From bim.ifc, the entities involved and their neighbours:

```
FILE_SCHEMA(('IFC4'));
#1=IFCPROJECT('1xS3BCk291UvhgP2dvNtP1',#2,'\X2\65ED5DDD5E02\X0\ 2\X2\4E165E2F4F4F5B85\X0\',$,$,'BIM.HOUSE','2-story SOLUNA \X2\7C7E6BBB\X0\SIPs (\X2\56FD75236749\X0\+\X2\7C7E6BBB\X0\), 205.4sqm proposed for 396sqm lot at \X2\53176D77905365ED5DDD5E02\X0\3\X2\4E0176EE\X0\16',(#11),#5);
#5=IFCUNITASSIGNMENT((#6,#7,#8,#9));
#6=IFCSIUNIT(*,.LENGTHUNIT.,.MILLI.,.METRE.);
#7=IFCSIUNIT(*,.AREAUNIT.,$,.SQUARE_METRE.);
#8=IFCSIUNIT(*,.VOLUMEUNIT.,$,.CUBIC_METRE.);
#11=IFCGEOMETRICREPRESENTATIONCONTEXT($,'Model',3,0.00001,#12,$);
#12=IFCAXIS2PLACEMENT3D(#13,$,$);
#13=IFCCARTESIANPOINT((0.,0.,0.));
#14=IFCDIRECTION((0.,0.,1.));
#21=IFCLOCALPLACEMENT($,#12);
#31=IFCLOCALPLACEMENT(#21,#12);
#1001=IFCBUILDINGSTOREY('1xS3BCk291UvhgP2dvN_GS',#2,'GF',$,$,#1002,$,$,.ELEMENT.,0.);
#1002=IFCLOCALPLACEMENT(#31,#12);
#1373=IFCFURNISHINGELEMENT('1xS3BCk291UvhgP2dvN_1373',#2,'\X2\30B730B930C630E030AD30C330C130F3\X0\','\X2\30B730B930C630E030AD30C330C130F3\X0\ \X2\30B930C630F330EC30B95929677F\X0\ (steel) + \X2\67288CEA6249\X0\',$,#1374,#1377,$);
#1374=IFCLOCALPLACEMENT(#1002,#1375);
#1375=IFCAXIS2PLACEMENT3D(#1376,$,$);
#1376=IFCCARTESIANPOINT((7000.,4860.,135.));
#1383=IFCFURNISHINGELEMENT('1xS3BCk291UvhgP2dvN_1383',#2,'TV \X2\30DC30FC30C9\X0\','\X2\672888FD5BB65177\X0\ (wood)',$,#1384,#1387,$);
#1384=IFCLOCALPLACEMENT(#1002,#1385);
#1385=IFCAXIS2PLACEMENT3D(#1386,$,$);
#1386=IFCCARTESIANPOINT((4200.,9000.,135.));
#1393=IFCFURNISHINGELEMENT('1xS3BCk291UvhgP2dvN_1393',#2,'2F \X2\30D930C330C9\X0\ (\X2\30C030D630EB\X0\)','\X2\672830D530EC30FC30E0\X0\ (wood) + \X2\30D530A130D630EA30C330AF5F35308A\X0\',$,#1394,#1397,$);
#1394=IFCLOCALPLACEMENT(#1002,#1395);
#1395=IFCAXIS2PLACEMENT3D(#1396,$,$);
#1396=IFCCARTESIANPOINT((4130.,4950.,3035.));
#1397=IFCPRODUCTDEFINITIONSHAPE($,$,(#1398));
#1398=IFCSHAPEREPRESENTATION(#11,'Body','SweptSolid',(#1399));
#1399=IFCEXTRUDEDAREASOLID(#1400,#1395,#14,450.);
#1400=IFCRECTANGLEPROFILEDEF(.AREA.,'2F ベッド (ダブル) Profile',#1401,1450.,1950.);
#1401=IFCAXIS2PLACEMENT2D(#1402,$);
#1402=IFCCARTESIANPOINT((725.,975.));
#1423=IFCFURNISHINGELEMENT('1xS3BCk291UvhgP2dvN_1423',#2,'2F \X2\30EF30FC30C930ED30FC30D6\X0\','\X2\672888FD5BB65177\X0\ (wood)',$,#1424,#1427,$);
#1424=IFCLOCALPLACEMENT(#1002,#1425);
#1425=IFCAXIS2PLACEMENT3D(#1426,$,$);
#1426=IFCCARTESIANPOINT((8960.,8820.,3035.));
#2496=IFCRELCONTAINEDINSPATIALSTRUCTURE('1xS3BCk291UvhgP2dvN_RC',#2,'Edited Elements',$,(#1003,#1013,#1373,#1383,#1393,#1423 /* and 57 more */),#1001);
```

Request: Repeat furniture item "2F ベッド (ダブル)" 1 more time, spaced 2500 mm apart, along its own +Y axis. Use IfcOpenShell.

```python
import ifcopenshell
import ifcopenshell.api.geometry
import ifcopenshell.api.root
import ifcopenshell.util.element
import ifcopenshell.util.placement
import ifcopenshell.util.unit

model = ifcopenshell.open("bim.ifc")
unit_scale = ifcopenshell.util.unit.calculate_unit_scale(model)


def reuse_history(source, copy):
    """copy_class also copies each property set's owner history, people and application; keep the originals."""
    for rel in copy.IsDefinedBy:
        if rel.is_a("IfcRelDefinesByProperties") and (history := rel.RelatingPropertyDefinition.OwnerHistory):
            rel.RelatingPropertyDefinition.OwnerHistory = source.OwnerHistory
            ifcopenshell.util.element.remove_deep2(model, history)


source = model.by_guid("1xS3BCk291UvhgP2dvN_1393")
base = ifcopenshell.util.placement.get_local_placement(source.ObjectPlacement)
step = base[:3, 1] * 2.5 / unit_scale

for i in range(1, 2):
    copy = ifcopenshell.api.root.copy_class(model, product=source)
    copy.Representation = ifcopenshell.util.element.copy_deep(
        model, source.Representation, exclude=["IfcGeometricRepresentationContext", "IfcRepresentationMap"]
    )
    reuse_history(source, copy)
    matrix = base.copy()
    matrix[:3, 3] += i * step
    print("added at", matrix[:3, 3].round(3) + 0.0)
    ifcopenshell.api.geometry.edit_object_placement(model, product=copy, matrix=matrix, is_si=False)

model.write("bim_edited.ifc")
```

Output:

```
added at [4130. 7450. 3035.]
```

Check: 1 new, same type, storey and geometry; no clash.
